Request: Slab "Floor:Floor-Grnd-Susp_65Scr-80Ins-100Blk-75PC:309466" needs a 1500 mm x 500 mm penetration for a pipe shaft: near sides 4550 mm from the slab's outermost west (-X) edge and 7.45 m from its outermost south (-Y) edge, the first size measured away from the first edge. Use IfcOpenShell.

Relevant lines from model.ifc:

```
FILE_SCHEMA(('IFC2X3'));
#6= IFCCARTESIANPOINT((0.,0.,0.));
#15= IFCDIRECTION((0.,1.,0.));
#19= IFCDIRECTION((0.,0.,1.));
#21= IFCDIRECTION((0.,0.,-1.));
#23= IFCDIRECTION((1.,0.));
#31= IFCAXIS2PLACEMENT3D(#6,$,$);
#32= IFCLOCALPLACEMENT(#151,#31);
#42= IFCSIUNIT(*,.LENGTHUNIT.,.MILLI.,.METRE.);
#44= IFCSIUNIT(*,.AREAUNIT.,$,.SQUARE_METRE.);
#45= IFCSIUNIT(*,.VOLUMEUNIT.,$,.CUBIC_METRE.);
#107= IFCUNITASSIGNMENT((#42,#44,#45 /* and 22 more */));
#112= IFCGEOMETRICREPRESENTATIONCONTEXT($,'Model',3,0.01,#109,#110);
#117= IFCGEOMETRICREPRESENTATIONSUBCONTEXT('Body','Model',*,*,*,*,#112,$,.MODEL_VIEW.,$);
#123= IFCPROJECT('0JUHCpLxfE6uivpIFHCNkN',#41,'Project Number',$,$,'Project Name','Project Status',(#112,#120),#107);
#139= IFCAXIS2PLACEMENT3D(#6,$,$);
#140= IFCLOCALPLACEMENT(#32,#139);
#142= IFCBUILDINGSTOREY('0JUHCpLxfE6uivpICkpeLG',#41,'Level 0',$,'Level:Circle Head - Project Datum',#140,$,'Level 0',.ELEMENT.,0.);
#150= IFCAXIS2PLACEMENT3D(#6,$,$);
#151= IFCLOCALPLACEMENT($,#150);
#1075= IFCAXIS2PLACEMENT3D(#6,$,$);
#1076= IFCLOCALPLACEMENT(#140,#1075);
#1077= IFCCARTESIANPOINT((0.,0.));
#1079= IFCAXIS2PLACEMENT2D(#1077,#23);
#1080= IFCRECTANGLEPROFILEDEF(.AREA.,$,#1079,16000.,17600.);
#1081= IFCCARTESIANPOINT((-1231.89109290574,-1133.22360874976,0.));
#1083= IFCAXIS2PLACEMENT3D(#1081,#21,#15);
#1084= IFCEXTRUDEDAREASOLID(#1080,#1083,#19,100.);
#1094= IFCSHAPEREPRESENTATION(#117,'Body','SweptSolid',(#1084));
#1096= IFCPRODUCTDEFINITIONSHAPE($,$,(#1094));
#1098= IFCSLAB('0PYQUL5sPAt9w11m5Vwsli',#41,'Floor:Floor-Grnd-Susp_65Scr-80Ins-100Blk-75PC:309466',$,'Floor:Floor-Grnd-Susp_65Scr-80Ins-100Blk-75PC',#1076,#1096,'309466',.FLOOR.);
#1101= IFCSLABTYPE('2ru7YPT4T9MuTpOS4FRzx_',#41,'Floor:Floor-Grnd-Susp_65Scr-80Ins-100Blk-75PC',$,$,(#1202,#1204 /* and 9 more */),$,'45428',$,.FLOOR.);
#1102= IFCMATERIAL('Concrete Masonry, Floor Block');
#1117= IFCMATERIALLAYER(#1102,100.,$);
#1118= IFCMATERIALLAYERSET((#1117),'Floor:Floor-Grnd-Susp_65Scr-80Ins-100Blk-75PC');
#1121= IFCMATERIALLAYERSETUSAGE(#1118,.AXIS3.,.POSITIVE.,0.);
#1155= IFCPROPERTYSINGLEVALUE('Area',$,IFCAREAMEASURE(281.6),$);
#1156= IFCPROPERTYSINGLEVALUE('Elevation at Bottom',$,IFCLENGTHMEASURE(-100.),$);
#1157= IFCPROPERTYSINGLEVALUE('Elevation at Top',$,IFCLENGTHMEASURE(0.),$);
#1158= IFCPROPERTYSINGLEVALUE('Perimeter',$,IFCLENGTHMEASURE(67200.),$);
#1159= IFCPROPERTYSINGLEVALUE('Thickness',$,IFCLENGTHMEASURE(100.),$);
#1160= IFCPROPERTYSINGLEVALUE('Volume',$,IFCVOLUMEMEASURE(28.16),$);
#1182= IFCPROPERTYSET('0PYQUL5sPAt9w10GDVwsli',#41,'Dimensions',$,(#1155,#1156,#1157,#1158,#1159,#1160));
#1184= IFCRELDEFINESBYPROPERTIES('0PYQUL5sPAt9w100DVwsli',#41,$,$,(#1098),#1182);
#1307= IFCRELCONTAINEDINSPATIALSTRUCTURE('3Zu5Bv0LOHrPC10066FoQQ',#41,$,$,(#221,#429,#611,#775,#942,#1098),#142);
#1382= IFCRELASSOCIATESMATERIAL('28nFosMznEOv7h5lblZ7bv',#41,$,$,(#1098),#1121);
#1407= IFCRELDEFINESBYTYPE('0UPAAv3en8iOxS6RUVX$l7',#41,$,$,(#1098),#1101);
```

```python
import numpy as np
import ifcopenshell
import ifcopenshell.api.feature
import ifcopenshell.api.geometry
import ifcopenshell.api.pset
import ifcopenshell.api.root
import ifcopenshell.geom
import ifcopenshell.util.element
import ifcopenshell.util.placement
import ifcopenshell.util.representation
import ifcopenshell.util.shape
import ifcopenshell.util.unit

model = ifcopenshell.open("model.ifc")
unit_scale = ifcopenshell.util.unit.calculate_unit_scale(model)
area_scale = ifcopenshell.util.unit.calculate_unit_scale(model, "AREAUNIT")
volume_scale = ifcopenshell.util.unit.calculate_unit_scale(model, "VOLUMEUNIT")
settings = ifcopenshell.geom.settings()


def volume(element):
    """Net volume in cubic metres, openings subtracted."""
    shape = ifcopenshell.geom.create_shape(settings, element)
    return ifcopenshell.util.shape.get_volume(shape.geometry)


slab = model.by_guid("0PYQUL5sPAt9w11m5Vwsli")
before = volume(slab)

# Extent in the slab's own axes, in metres. The edges named are its -X and -Y sides.
slab_shape = ifcopenshell.geom.create_shape(settings, slab)
vertices = ifcopenshell.util.shape.get_vertices(slab_shape.geometry)
x_min, y_min, bottom = vertices.min(axis=0)
top = vertices[:, 2].max()

opening = ifcopenshell.api.root.create_entity(model, ifc_class="IfcOpeningElement", name="Pipe shaft opening")
context = ifcopenshell.util.representation.get_context(model, "Model", "Body", "MODEL_VIEW")
width, depth = 1.5, 0.5
outline = [(0.0, 0.0), (width, 0.0), (width, depth), (0.0, depth), (0.0, 0.0)]
# Overshoot both faces by 50 mm so the cut is clean.
shape = ifcopenshell.api.geometry.add_slab_representation(
    model, context=context, depth=top - bottom + 0.1, polyline=outline
)
ifcopenshell.api.geometry.assign_representation(model, product=opening, representation=shape)

matrix = ifcopenshell.util.placement.get_local_placement(slab.ObjectPlacement)
matrix[:, 3] = matrix @ np.append(np.array([x_min + 4.55, y_min + 7.45, bottom - 0.05]) / unit_scale, 1.0)
ifcopenshell.api.geometry.edit_object_placement(model, product=opening, matrix=matrix, is_si=False)
ifcopenshell.api.feature.add_feature(model, feature=opening, element=slab)

after = volume(slab)

# Update the slab's stored quantities.
pset = model.by_id(ifcopenshell.util.element.get_pset(slab, "Dimensions", should_inherit=False)["id"])
ifcopenshell.api.pset.edit_pset(model, pset=pset, properties={
    "Area": model.create_entity("IfcAreaMeasure", after / (top - bottom) / area_scale),
    "Volume": model.create_entity("IfcVolumeMeasure", after / volume_scale),
})

print(f"slab volume {before:.3f} -> {after:.3f} m3")

model.write("model_edited.ifc")
```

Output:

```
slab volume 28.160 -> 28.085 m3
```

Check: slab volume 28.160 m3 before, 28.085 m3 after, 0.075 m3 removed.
